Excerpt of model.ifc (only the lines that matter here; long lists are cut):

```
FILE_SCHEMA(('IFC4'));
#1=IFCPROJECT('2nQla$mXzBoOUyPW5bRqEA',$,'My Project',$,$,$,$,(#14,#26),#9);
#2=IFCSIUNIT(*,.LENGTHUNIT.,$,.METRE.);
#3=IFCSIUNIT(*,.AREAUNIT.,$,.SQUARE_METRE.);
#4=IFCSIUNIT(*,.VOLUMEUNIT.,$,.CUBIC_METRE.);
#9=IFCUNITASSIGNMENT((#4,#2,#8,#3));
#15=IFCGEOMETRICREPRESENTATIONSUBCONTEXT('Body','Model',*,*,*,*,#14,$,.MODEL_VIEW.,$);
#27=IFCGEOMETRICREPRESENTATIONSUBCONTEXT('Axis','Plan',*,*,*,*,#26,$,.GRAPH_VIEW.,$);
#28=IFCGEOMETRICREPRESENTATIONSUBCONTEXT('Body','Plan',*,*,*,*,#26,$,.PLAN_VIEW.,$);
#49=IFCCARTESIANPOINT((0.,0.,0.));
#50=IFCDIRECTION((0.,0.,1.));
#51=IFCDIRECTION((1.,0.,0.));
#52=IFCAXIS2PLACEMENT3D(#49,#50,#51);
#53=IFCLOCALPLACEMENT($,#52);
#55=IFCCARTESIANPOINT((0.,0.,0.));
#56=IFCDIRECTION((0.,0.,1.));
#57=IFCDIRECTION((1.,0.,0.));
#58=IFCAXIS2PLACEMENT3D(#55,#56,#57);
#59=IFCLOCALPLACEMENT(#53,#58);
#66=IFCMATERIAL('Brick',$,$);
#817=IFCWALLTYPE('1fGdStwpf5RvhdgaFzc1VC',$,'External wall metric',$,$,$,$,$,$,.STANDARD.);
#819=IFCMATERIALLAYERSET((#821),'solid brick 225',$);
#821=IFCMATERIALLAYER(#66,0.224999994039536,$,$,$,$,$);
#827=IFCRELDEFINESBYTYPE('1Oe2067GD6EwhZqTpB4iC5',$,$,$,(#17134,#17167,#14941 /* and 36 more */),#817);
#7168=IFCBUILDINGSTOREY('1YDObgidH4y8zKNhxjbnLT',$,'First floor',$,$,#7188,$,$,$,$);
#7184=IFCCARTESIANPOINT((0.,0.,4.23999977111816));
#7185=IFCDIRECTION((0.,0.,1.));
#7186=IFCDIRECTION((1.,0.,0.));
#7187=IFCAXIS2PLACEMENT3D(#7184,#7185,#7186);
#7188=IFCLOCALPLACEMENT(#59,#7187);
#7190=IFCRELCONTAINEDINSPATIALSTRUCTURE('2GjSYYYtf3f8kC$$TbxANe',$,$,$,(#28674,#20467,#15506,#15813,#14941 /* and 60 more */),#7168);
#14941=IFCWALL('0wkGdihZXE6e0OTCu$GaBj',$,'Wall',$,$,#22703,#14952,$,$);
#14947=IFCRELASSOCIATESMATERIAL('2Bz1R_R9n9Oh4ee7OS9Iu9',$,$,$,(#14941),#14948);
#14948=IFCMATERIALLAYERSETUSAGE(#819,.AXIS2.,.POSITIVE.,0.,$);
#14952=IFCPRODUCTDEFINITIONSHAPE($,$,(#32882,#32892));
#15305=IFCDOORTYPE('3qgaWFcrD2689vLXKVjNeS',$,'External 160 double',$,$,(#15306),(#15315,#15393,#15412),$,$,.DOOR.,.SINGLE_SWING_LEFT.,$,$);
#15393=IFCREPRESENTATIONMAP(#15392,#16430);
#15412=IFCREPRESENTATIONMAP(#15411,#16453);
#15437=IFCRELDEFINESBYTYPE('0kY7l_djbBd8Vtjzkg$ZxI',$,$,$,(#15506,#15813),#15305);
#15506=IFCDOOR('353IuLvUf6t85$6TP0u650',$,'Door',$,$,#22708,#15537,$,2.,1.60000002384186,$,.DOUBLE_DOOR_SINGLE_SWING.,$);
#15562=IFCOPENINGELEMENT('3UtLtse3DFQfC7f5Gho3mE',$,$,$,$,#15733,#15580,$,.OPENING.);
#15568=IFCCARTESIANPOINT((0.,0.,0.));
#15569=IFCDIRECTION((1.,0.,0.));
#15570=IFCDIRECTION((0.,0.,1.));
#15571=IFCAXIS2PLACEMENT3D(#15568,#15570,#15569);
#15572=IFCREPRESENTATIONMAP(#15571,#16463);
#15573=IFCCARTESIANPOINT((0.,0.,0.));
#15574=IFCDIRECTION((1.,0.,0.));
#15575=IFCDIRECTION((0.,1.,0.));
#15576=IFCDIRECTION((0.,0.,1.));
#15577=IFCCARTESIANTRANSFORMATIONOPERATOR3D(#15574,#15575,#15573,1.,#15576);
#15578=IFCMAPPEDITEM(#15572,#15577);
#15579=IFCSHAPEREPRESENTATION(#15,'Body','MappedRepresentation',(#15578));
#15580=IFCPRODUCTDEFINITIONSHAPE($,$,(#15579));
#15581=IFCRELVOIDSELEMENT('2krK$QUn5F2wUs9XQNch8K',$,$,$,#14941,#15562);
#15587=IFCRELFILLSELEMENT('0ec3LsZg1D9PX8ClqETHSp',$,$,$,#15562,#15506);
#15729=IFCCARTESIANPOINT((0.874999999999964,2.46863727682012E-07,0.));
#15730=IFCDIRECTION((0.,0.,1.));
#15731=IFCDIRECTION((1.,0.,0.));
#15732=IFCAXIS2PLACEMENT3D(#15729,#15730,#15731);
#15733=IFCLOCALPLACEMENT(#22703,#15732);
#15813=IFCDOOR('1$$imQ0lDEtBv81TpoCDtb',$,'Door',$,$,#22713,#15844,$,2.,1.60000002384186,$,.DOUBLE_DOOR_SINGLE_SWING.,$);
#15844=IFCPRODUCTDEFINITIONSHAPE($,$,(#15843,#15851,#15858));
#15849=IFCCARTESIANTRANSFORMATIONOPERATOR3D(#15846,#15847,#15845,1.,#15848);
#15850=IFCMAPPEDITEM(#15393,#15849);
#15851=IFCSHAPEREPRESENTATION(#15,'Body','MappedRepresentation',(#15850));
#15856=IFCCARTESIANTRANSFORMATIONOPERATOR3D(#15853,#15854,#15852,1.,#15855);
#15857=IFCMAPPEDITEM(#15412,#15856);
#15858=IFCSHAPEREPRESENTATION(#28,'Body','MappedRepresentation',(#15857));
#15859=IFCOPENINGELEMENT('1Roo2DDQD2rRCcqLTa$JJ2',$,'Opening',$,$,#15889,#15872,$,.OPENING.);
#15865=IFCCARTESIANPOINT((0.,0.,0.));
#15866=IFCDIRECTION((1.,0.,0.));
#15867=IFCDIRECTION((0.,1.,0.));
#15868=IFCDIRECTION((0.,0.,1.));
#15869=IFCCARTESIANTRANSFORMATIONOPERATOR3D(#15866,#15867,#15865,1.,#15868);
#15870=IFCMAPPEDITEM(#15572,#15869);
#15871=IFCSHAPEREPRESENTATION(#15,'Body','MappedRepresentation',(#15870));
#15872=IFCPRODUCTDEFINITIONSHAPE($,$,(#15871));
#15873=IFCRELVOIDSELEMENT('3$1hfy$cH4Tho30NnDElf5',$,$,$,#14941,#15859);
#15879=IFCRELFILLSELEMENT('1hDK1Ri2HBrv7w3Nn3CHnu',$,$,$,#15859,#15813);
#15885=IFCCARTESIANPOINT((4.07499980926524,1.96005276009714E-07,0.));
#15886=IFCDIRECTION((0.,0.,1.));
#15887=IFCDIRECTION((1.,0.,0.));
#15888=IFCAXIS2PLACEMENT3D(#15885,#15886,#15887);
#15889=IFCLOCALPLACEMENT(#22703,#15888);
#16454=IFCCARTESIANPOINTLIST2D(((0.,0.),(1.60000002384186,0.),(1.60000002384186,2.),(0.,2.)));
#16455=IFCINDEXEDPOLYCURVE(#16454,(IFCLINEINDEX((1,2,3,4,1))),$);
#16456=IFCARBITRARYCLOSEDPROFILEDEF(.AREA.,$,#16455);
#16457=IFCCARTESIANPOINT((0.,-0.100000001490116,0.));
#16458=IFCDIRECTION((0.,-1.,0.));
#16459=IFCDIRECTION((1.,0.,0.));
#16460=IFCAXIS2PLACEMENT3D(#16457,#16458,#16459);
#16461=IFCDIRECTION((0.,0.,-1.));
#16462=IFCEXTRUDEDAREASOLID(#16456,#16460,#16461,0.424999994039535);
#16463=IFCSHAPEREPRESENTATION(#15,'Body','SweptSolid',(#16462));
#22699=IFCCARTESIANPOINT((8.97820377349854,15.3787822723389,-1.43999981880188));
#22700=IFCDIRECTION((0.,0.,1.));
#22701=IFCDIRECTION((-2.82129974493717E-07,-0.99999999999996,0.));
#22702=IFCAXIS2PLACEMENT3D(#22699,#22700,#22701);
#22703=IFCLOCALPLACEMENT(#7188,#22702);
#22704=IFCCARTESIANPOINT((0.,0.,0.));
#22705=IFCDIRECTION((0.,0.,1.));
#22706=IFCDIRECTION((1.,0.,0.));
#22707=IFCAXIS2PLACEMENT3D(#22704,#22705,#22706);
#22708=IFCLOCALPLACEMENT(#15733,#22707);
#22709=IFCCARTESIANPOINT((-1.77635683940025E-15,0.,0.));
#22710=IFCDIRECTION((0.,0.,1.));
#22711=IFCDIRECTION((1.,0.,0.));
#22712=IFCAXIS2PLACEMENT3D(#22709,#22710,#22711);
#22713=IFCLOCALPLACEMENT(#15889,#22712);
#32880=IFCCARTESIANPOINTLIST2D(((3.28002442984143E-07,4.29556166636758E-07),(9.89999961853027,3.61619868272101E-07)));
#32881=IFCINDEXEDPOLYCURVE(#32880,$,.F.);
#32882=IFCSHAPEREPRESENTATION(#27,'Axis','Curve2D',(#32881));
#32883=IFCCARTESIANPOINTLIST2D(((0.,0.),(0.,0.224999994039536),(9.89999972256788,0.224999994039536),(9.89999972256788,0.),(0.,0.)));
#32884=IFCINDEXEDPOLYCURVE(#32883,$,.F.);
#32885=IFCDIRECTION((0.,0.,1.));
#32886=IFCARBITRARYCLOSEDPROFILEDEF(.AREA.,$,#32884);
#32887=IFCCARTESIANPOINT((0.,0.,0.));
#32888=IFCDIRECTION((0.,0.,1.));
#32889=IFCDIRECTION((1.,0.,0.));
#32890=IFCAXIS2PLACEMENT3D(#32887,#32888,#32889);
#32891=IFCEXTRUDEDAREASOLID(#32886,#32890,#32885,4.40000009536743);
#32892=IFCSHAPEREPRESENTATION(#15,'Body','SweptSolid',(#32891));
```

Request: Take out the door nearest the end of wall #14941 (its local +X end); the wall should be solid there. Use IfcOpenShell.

```python
import ifcopenshell
import ifcopenshell.api.feature
import ifcopenshell.api.root
import ifcopenshell.geom
import ifcopenshell.util.shape

model = ifcopenshell.open("model.ifc")
settings = ifcopenshell.geom.settings()


def volume(element):
    """Net volume in cubic metres, openings subtracted."""
    shape = ifcopenshell.geom.create_shape(settings, element)
    return ifcopenshell.util.shape.get_volume(shape.geometry)


door = model.by_guid("1$$imQ0lDEtBv81TpoCDtb")
opening = door.FillsVoids[0].RelatingOpeningElement
wall = opening.VoidsElements[0].RelatingBuildingElement
before = volume(wall)

ifcopenshell.api.root.remove_product(model, product=door)
ifcopenshell.api.feature.remove_feature(model, feature=opening)

after = volume(wall)

print(f"wall volume {before:.3f} -> {after:.3f} m3")

model.write("model_updated.ifc")
```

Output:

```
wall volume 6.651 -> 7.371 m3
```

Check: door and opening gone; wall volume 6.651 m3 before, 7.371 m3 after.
